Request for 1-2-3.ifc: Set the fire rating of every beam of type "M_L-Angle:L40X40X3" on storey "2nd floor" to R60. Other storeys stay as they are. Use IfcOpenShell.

First a look at what the model holds.

```python
import ifcopenshell
import ifcopenshell.util.element

model = ifcopenshell.open("1-2-3.ifc")
print(model.schema)
storey = next(s for s in model.by_type("IfcBuildingStorey") if s.Name == "2nd floor")
beams = [e for e in ifcopenshell.util.element.get_decomposition(storey) if e.is_a("IfcBeam")]
seen = {}
for e in beams:
    element_type = ifcopenshell.util.element.get_type(e)
    key = (element_type.Name if element_type != e and element_type else None, ifcopenshell.util.element.get_pset(e, "Pset_BeamCommon", "FireRating"))
    seen[key] = seen.get(key, 0) + 1
for (name, value), count in sorted(seen.items(), key=str):
    print(count, "x", name, "|", value)
```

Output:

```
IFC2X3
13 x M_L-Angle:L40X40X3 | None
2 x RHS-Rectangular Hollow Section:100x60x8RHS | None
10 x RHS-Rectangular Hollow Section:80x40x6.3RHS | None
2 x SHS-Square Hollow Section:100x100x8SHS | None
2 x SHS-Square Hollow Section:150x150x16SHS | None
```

```python
import ifcopenshell
import ifcopenshell.api.pset
import ifcopenshell.util.element

model = ifcopenshell.open("1-2-3.ifc")

storey = next(s for s in model.by_type("IfcBuildingStorey") if s.Name == "2nd floor")
beams = [e for e in ifcopenshell.util.element.get_decomposition(storey) if e.is_a("IfcBeam")]

count = 0
for e in beams:
    element_type = ifcopenshell.util.element.get_type(e)
    if element_type in (None, e) or element_type.Name != "M_L-Angle:L40X40X3":
        continue
    # add_pset returns the element's existing set when there is one.
    pset = ifcopenshell.api.pset.add_pset(model, product=e, name="Pset_BeamCommon")
    ifcopenshell.api.pset.edit_pset(model, pset=pset, properties={"FireRating": "R60"})
    count += 1

print(count, "beams updated")

model.write("1-2-3_updated.ifc")
```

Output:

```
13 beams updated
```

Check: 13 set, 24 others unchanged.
